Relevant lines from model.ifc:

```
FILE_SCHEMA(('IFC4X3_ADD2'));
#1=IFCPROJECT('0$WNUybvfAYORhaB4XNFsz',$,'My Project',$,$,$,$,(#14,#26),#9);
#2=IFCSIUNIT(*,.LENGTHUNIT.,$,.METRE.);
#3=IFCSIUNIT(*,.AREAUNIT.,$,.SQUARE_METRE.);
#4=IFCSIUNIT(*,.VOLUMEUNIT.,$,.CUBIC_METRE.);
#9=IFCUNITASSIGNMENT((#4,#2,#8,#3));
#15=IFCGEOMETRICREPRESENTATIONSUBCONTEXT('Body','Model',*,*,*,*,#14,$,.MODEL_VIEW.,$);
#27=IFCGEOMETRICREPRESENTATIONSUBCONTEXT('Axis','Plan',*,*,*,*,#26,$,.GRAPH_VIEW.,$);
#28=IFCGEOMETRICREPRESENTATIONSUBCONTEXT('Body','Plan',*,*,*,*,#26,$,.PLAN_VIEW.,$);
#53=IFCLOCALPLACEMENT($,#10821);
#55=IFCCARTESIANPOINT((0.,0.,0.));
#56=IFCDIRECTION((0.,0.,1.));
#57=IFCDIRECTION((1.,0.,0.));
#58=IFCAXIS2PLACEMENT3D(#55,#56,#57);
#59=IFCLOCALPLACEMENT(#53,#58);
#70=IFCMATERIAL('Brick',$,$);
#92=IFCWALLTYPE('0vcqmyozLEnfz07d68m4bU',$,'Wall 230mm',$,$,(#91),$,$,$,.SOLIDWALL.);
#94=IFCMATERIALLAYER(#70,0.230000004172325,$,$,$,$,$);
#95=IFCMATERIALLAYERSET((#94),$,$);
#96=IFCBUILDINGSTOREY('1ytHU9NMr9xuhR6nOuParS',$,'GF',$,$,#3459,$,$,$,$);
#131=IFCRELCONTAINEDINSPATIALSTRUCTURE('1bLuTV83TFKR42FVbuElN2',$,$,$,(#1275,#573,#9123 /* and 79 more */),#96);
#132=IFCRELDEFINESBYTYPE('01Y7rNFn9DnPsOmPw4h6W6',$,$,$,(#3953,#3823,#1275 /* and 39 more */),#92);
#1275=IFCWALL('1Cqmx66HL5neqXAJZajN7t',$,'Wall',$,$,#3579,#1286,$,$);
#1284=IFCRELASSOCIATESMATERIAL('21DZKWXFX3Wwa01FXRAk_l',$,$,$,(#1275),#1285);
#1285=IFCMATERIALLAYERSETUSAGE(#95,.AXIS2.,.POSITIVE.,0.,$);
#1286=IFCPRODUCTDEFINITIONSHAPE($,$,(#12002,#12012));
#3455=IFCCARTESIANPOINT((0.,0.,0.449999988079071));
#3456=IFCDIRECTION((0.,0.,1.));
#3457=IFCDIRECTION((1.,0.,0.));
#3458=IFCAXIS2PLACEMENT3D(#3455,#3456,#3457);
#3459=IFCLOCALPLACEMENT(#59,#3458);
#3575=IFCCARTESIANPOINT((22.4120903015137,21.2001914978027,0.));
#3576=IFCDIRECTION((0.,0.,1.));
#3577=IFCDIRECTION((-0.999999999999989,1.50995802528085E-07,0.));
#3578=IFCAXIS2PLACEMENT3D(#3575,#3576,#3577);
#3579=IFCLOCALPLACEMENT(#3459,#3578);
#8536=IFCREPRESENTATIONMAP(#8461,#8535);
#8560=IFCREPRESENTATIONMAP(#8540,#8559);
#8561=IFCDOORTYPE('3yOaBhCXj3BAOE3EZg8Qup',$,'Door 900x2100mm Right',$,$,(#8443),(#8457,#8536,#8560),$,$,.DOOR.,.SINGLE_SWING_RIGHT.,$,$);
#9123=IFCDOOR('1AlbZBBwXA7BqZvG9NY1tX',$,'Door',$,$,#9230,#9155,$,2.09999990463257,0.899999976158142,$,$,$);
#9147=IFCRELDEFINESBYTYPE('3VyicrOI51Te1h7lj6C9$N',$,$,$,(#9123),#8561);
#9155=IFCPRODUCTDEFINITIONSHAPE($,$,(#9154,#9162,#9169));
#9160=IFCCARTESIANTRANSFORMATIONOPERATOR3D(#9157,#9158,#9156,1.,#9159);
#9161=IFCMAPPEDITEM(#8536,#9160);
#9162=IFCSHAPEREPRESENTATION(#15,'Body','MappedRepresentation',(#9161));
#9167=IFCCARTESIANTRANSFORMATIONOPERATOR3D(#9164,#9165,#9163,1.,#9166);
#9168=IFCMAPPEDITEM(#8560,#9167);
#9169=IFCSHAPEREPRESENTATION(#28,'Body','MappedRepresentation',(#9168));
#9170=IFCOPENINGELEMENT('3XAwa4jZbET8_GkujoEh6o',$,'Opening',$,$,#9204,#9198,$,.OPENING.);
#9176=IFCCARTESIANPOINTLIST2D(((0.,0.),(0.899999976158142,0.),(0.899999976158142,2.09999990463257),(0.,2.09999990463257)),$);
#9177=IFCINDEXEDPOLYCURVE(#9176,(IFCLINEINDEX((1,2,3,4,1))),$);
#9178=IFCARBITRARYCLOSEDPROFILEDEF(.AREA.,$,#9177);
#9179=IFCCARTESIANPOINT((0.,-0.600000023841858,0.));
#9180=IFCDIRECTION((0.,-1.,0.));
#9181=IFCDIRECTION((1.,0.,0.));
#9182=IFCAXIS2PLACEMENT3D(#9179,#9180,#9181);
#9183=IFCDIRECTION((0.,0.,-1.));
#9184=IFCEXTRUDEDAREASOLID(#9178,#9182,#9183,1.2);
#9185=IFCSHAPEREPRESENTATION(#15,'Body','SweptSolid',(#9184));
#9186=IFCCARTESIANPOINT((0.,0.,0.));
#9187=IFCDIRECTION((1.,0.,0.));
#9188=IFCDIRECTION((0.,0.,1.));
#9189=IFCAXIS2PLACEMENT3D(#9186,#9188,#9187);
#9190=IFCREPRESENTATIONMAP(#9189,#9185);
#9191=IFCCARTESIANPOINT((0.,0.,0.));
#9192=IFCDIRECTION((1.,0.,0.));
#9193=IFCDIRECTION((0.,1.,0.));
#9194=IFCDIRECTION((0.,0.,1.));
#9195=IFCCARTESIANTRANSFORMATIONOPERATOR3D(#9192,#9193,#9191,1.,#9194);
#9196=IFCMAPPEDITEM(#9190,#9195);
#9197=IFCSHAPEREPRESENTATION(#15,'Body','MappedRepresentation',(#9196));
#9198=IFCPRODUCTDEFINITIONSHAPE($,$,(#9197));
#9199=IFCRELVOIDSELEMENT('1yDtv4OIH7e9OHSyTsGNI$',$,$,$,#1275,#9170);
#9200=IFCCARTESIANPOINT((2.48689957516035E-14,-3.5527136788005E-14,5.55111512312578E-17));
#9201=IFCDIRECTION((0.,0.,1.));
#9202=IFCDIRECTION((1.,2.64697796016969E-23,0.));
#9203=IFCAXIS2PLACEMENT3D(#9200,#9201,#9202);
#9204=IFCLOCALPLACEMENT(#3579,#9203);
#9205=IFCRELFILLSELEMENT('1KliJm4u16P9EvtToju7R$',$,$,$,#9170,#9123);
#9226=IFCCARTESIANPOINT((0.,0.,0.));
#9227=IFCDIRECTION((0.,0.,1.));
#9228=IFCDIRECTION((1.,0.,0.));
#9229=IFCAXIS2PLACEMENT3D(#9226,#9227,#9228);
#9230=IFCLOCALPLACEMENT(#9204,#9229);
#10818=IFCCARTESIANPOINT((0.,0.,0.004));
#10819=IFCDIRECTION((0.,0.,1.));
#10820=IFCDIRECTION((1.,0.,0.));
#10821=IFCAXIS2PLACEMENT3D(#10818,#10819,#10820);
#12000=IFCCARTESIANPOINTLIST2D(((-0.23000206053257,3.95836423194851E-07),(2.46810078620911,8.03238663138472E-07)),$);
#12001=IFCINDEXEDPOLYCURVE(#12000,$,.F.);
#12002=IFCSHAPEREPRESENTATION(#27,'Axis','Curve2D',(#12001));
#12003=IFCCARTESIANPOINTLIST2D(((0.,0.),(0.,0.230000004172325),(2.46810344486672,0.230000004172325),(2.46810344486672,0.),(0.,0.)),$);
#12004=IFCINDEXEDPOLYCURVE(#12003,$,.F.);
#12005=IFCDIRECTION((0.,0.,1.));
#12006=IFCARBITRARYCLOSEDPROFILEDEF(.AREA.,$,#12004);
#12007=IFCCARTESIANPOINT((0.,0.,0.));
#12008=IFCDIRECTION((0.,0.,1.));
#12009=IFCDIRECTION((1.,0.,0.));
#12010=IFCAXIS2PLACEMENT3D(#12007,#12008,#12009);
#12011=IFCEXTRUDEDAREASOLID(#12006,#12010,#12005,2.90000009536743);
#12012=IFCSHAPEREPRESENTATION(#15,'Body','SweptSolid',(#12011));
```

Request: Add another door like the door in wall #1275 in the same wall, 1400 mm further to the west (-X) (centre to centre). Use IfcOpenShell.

```python
import ifcopenshell
import ifcopenshell.api.feature
import ifcopenshell.api.geometry
import ifcopenshell.api.root
import ifcopenshell.geom
import ifcopenshell.util.element
import ifcopenshell.util.placement
import ifcopenshell.util.shape

model = ifcopenshell.open("model.ifc")
settings = ifcopenshell.geom.settings()


def volume(element):
    """Net volume in cubic metres, openings subtracted."""
    shape = ifcopenshell.geom.create_shape(settings, element)
    return ifcopenshell.util.shape.get_volume(shape.geometry)


door = model.by_id(9123)
opening = door.FillsVoids[0].RelatingOpeningElement
wall = opening.VoidsElements[0].RelatingBuildingElement
before = volume(wall)
shift = ifcopenshell.util.placement.get_local_placement(wall.ObjectPlacement)[:3, 0] * 1.4

# copy_class copies the void relationship, type, container and properties, but no geometry.
new_opening = ifcopenshell.api.root.copy_class(model, product=opening)
new_opening.Representation = ifcopenshell.util.element.copy_deep(
    model, opening.Representation, exclude=["IfcGeometricRepresentationContext", "IfcRepresentationMap"]
)
new_door = ifcopenshell.api.root.copy_class(model, product=door)
new_door.Representation = ifcopenshell.util.element.copy_deep(
    model, door.Representation, exclude=["IfcGeometricRepresentationContext", "IfcRepresentationMap"]
)
ifcopenshell.api.feature.add_filling(model, opening=new_opening, element=new_door)

for old, new in ((opening, new_opening), (door, new_door)):
    matrix = ifcopenshell.util.placement.get_local_placement(old.ObjectPlacement)
    matrix[:3, 3] += shift
    ifcopenshell.api.geometry.edit_object_placement(model, product=new, matrix=matrix, is_si=False)

after = volume(wall)

print(f"wall volume {before:.3f} -> {after:.3f} m3")

model.write("model_rev.ifc")
```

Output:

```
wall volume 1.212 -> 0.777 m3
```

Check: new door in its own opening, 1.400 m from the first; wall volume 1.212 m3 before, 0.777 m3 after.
